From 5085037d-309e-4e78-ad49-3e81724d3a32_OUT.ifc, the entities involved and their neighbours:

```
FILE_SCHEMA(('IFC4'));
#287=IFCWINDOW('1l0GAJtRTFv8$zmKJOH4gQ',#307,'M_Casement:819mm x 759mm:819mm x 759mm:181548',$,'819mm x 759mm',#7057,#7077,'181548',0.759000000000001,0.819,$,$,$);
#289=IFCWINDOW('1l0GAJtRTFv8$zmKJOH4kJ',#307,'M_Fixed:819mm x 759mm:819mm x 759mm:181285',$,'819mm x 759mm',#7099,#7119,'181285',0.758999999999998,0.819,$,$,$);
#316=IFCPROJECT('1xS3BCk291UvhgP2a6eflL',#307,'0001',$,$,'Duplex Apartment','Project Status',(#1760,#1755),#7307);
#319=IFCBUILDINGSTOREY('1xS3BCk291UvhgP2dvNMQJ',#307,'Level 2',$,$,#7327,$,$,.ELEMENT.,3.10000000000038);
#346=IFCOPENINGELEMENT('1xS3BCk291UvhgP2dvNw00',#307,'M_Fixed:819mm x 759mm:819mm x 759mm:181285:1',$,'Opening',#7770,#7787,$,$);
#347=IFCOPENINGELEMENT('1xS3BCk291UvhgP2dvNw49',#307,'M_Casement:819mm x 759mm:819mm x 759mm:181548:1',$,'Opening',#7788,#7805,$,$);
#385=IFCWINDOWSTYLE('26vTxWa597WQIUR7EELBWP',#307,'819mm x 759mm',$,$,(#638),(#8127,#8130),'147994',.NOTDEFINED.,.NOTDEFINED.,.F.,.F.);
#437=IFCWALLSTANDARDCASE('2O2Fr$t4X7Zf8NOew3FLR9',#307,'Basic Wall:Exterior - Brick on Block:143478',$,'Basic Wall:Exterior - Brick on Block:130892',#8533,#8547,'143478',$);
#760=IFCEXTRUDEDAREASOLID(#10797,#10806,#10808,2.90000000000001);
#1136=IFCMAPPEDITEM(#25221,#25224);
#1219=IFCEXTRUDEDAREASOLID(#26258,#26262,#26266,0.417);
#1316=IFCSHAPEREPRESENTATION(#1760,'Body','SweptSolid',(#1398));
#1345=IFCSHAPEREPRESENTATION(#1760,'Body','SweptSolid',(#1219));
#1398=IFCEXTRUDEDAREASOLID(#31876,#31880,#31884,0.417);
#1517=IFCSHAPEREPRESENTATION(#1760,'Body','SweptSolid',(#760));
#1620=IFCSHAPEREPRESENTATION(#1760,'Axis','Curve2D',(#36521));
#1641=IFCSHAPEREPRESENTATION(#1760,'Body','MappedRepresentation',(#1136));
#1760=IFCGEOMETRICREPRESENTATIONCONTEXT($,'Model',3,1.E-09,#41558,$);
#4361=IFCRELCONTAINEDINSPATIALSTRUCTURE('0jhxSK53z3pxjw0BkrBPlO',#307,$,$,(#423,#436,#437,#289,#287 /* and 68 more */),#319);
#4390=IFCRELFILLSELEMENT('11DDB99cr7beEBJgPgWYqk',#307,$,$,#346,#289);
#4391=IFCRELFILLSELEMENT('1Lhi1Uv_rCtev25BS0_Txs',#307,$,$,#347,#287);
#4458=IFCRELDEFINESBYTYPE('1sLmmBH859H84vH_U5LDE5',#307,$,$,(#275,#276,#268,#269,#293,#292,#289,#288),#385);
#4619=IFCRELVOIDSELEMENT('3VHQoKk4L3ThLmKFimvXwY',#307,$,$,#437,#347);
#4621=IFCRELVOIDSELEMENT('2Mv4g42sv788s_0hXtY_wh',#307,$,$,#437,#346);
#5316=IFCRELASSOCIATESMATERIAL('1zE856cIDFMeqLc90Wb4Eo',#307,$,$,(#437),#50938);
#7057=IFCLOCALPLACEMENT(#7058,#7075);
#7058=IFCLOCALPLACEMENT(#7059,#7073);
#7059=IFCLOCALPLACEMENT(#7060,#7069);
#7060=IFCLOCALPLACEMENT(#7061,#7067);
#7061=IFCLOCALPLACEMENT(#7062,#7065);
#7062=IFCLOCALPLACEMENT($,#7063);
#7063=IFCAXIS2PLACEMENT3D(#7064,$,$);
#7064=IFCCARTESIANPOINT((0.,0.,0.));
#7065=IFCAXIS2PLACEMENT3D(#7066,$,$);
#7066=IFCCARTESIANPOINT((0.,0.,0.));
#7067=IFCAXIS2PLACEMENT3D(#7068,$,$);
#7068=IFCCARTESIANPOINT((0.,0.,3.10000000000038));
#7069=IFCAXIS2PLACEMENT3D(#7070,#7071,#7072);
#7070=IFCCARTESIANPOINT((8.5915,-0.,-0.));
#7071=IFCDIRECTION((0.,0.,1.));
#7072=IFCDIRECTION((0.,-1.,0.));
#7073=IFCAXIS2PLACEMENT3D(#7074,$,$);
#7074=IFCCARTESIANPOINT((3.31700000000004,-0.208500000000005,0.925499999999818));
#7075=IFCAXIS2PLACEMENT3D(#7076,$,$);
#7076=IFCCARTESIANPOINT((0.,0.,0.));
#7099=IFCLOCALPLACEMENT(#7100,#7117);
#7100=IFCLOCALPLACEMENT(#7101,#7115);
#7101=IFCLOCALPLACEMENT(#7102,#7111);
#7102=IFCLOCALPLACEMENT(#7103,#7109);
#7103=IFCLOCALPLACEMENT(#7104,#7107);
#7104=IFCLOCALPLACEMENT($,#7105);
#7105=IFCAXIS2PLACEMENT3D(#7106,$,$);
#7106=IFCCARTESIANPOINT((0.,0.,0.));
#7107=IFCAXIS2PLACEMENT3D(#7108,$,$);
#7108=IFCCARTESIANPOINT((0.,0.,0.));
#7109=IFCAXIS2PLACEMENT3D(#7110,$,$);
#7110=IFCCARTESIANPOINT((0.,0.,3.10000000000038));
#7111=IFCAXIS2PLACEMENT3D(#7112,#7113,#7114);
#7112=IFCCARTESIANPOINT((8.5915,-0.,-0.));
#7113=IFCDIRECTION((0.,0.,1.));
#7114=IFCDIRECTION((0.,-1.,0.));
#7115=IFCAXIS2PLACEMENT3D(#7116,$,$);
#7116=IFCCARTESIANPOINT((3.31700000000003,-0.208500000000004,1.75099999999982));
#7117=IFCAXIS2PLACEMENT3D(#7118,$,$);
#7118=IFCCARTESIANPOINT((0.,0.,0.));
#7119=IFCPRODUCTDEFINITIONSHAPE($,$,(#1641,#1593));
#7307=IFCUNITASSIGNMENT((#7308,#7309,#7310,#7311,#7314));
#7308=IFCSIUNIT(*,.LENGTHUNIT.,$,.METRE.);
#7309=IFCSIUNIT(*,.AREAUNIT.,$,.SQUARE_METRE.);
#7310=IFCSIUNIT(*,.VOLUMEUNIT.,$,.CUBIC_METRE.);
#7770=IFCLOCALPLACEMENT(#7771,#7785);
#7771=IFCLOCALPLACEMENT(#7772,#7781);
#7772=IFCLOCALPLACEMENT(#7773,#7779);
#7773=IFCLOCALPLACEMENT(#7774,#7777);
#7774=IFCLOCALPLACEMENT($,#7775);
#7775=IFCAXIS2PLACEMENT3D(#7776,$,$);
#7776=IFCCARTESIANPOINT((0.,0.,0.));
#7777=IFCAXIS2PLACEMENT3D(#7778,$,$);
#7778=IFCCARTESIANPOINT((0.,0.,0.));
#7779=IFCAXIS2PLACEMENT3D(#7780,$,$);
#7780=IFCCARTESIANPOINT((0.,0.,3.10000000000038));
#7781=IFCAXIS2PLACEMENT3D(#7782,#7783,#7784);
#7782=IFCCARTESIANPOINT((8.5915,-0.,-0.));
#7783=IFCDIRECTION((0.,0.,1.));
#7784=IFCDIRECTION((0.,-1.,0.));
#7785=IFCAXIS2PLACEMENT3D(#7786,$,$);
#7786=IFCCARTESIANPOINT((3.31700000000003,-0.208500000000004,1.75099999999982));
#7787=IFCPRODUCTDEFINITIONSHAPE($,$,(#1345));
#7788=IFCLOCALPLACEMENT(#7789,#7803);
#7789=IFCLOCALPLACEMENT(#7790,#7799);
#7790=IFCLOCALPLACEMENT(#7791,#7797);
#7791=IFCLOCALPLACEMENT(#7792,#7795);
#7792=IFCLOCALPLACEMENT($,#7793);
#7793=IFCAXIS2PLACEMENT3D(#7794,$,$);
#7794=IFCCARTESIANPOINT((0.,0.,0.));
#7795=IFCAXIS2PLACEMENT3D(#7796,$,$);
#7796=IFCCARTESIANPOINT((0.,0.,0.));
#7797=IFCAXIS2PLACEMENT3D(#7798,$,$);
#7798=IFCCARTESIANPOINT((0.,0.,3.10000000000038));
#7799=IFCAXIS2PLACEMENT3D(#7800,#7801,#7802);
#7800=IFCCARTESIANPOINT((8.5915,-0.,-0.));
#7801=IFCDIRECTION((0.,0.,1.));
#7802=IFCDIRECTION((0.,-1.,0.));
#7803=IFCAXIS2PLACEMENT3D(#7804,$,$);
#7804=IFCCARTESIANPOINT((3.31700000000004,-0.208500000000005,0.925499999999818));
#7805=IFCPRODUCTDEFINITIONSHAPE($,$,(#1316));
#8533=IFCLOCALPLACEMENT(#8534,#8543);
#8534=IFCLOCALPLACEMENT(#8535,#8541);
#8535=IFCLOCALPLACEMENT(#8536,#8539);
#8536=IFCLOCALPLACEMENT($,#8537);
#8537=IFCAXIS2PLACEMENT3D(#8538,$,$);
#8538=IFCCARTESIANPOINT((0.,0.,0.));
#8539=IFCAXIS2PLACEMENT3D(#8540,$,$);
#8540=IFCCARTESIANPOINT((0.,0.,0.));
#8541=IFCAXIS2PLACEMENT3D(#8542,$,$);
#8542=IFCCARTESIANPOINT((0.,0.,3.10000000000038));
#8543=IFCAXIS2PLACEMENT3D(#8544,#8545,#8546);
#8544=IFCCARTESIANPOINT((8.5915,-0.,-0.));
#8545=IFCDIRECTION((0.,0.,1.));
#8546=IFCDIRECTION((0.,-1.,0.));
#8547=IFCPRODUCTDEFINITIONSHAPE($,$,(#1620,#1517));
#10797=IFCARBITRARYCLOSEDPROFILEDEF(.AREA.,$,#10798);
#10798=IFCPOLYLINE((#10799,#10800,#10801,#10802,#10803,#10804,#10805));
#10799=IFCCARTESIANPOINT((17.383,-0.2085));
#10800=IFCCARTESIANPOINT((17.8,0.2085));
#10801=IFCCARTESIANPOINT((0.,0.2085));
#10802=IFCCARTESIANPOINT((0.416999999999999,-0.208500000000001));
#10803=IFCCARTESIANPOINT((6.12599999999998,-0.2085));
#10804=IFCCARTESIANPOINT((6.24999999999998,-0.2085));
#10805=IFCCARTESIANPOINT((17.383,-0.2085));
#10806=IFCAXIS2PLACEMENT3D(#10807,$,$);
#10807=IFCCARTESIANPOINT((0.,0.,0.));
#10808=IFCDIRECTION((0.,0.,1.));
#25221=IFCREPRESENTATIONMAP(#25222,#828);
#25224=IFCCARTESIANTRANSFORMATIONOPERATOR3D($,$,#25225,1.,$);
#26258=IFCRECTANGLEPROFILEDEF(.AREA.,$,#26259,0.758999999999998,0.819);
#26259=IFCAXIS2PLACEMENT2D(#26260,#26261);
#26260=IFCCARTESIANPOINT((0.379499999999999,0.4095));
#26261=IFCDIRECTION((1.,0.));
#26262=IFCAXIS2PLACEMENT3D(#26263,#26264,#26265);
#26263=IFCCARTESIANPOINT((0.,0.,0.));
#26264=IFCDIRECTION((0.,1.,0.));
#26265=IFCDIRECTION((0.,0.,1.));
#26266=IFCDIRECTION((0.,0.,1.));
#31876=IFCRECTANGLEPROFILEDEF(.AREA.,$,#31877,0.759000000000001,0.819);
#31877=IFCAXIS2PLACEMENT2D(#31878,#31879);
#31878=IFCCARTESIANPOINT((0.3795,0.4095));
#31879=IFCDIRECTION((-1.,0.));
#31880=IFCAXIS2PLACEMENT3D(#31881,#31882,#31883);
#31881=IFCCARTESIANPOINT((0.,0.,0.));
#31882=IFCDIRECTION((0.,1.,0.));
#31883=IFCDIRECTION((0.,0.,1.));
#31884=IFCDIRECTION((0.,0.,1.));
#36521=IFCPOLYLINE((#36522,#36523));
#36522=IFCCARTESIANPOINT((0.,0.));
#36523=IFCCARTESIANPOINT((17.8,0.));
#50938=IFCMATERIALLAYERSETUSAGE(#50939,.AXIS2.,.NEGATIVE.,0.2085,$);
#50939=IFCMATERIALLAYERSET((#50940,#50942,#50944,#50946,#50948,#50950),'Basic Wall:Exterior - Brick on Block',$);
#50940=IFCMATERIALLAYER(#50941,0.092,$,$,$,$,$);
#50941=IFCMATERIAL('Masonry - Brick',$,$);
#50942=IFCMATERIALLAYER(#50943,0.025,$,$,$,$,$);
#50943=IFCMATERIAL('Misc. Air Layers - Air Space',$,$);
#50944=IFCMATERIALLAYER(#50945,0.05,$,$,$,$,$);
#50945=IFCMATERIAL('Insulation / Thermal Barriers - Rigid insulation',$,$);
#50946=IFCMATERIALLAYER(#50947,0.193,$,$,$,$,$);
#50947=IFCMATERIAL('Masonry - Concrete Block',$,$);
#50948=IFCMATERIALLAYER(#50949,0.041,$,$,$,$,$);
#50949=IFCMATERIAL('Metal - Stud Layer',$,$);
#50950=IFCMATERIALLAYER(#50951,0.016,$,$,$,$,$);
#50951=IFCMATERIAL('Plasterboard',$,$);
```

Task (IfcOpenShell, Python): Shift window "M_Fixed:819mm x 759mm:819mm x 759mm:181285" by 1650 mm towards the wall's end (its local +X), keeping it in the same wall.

```python
import ifcopenshell
import ifcopenshell.api.geometry
import ifcopenshell.util.placement
import ifcopenshell.util.unit

model = ifcopenshell.open("5085037d-309e-4e78-ad49-3e81724d3a32_OUT.ifc")
unit_scale = ifcopenshell.util.unit.calculate_unit_scale(model)

window = model.by_guid("1l0GAJtRTFv8$zmKJOH4kJ")
opening = window.FillsVoids[0].RelatingOpeningElement
wall = opening.VoidsElements[0].RelatingBuildingElement

wall_matrix = ifcopenshell.util.placement.get_local_placement(wall.ObjectPlacement)
shift = wall_matrix[:3, 0] * 1.65 / unit_scale
before = ifcopenshell.util.placement.get_local_placement(window.ObjectPlacement)[:3, 3].copy()

# The window is not placed relative to its opening, so move both.
for product in (opening, window):
    matrix = ifcopenshell.util.placement.get_local_placement(product.ObjectPlacement)
    matrix[:3, 3] += shift
    ifcopenshell.api.geometry.edit_object_placement(model, product=product, matrix=matrix, is_si=False)

after = ifcopenshell.util.placement.get_local_placement(window.ObjectPlacement)[:3, 3]
print("window moved by", (after - before).round(3) + 0.0)

model.write("5085037d-309e-4e78-ad49-3e81724d3a32_OUT_edited.ifc")
```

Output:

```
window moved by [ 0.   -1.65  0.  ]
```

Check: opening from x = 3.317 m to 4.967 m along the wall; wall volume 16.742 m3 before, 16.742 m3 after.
